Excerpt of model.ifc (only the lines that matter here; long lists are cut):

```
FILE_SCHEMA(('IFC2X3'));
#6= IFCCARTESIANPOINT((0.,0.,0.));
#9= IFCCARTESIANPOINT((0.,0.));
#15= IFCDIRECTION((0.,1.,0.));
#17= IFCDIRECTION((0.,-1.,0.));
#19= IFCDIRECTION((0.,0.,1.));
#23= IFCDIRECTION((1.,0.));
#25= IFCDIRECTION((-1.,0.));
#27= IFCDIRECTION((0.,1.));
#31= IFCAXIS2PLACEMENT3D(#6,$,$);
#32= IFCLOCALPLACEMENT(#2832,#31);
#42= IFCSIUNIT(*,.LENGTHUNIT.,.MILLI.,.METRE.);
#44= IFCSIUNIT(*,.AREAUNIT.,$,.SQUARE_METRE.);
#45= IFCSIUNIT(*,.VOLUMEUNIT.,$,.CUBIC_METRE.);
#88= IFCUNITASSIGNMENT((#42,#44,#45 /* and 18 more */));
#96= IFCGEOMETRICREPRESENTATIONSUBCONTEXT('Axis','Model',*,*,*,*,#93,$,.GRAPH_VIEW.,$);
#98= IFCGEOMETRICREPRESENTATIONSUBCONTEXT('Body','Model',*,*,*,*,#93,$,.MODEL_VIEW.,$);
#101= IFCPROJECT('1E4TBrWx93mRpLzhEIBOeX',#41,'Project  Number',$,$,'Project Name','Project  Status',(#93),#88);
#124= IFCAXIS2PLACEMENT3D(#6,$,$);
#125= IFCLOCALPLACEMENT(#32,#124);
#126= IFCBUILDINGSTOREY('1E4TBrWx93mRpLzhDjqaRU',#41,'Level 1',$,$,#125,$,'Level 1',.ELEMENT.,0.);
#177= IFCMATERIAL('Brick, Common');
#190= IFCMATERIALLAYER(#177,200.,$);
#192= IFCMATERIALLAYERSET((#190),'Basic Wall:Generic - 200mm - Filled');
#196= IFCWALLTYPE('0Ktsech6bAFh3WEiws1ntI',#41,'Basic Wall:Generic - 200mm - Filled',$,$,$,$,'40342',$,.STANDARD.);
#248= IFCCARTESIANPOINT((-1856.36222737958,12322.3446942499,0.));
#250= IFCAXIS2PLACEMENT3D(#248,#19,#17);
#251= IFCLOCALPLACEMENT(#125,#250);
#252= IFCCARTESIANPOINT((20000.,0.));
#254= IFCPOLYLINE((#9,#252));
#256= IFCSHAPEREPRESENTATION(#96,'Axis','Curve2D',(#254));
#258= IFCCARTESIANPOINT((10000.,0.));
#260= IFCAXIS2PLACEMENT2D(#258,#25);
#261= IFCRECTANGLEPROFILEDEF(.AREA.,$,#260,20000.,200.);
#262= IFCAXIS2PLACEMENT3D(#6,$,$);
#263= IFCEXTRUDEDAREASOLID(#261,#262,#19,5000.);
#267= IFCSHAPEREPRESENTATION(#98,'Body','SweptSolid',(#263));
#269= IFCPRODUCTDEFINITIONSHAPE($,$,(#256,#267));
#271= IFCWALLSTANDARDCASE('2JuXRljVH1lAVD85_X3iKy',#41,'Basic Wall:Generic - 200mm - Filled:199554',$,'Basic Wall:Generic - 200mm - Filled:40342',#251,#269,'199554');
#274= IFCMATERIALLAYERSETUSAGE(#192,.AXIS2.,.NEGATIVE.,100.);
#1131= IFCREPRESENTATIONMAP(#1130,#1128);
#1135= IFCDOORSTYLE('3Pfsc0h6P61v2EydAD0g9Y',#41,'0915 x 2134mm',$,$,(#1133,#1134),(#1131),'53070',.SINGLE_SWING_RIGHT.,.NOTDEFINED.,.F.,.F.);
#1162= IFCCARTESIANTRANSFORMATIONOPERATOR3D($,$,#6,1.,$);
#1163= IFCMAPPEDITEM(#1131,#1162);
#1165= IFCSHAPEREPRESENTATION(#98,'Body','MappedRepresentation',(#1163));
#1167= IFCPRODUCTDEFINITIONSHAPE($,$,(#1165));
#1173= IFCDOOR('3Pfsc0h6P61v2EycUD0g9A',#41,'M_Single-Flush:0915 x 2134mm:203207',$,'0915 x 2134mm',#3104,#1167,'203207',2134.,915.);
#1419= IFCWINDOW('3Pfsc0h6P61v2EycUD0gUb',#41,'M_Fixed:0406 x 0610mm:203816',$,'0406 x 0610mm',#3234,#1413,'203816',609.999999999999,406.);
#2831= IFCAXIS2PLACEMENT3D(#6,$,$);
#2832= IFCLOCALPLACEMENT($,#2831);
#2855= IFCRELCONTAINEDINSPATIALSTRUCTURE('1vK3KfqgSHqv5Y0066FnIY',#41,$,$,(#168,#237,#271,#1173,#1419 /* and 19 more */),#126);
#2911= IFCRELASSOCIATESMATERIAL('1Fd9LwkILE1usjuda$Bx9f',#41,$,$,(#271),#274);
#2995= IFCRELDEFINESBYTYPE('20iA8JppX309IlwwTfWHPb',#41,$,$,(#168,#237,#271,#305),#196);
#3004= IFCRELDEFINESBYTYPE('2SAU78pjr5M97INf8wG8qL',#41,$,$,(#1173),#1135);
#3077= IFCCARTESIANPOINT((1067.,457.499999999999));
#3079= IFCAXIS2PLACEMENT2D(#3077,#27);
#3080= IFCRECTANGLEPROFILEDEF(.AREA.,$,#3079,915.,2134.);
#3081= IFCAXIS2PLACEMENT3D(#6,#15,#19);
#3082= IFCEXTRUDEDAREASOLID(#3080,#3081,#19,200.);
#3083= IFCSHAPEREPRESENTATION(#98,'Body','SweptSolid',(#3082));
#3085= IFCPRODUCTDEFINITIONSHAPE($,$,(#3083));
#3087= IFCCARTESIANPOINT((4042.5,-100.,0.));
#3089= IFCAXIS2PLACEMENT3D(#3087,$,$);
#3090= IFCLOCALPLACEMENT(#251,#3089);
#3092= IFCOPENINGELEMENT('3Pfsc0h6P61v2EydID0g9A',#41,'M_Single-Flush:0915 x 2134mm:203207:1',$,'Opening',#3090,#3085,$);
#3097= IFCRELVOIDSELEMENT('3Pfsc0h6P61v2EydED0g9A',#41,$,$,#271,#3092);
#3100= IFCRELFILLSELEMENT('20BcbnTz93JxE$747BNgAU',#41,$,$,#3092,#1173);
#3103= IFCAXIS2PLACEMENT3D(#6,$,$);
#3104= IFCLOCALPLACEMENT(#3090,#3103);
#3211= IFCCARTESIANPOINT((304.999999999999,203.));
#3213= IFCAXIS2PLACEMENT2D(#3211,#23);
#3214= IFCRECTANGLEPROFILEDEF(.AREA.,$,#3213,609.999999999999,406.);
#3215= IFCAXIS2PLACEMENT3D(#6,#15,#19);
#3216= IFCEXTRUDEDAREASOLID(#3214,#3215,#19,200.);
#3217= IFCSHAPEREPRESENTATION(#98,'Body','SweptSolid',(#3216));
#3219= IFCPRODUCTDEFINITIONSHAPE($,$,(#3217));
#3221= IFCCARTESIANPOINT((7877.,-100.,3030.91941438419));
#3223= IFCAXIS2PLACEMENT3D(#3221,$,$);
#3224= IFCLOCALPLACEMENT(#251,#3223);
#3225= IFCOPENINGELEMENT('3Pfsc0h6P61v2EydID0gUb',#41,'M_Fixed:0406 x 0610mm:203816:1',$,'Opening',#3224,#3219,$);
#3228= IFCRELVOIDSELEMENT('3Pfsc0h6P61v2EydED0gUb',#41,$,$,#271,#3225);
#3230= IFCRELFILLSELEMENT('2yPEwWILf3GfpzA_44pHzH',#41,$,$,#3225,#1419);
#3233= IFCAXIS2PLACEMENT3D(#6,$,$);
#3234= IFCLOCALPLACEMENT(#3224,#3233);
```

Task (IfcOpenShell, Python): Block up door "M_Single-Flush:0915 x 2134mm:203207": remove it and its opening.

```python
import ifcopenshell
import ifcopenshell.api.feature
import ifcopenshell.api.root
import ifcopenshell.geom
import ifcopenshell.util.shape

model = ifcopenshell.open("model.ifc")
settings = ifcopenshell.geom.settings()


def volume(element):
    """Net volume in cubic metres, openings subtracted."""
    shape = ifcopenshell.geom.create_shape(settings, element)
    return ifcopenshell.util.shape.get_volume(shape.geometry)


door = model.by_guid("3Pfsc0h6P61v2EycUD0g9A")
opening = door.FillsVoids[0].RelatingOpeningElement
wall = opening.VoidsElements[0].RelatingBuildingElement
before = volume(wall)

ifcopenshell.api.root.remove_product(model, product=door)
ifcopenshell.api.feature.remove_feature(model, feature=opening)

after = volume(wall)

print(f"wall volume {before:.3f} -> {after:.3f} m3")

model.write("model_updated.ifc")
```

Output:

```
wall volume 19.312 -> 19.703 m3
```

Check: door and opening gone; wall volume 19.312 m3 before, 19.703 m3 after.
